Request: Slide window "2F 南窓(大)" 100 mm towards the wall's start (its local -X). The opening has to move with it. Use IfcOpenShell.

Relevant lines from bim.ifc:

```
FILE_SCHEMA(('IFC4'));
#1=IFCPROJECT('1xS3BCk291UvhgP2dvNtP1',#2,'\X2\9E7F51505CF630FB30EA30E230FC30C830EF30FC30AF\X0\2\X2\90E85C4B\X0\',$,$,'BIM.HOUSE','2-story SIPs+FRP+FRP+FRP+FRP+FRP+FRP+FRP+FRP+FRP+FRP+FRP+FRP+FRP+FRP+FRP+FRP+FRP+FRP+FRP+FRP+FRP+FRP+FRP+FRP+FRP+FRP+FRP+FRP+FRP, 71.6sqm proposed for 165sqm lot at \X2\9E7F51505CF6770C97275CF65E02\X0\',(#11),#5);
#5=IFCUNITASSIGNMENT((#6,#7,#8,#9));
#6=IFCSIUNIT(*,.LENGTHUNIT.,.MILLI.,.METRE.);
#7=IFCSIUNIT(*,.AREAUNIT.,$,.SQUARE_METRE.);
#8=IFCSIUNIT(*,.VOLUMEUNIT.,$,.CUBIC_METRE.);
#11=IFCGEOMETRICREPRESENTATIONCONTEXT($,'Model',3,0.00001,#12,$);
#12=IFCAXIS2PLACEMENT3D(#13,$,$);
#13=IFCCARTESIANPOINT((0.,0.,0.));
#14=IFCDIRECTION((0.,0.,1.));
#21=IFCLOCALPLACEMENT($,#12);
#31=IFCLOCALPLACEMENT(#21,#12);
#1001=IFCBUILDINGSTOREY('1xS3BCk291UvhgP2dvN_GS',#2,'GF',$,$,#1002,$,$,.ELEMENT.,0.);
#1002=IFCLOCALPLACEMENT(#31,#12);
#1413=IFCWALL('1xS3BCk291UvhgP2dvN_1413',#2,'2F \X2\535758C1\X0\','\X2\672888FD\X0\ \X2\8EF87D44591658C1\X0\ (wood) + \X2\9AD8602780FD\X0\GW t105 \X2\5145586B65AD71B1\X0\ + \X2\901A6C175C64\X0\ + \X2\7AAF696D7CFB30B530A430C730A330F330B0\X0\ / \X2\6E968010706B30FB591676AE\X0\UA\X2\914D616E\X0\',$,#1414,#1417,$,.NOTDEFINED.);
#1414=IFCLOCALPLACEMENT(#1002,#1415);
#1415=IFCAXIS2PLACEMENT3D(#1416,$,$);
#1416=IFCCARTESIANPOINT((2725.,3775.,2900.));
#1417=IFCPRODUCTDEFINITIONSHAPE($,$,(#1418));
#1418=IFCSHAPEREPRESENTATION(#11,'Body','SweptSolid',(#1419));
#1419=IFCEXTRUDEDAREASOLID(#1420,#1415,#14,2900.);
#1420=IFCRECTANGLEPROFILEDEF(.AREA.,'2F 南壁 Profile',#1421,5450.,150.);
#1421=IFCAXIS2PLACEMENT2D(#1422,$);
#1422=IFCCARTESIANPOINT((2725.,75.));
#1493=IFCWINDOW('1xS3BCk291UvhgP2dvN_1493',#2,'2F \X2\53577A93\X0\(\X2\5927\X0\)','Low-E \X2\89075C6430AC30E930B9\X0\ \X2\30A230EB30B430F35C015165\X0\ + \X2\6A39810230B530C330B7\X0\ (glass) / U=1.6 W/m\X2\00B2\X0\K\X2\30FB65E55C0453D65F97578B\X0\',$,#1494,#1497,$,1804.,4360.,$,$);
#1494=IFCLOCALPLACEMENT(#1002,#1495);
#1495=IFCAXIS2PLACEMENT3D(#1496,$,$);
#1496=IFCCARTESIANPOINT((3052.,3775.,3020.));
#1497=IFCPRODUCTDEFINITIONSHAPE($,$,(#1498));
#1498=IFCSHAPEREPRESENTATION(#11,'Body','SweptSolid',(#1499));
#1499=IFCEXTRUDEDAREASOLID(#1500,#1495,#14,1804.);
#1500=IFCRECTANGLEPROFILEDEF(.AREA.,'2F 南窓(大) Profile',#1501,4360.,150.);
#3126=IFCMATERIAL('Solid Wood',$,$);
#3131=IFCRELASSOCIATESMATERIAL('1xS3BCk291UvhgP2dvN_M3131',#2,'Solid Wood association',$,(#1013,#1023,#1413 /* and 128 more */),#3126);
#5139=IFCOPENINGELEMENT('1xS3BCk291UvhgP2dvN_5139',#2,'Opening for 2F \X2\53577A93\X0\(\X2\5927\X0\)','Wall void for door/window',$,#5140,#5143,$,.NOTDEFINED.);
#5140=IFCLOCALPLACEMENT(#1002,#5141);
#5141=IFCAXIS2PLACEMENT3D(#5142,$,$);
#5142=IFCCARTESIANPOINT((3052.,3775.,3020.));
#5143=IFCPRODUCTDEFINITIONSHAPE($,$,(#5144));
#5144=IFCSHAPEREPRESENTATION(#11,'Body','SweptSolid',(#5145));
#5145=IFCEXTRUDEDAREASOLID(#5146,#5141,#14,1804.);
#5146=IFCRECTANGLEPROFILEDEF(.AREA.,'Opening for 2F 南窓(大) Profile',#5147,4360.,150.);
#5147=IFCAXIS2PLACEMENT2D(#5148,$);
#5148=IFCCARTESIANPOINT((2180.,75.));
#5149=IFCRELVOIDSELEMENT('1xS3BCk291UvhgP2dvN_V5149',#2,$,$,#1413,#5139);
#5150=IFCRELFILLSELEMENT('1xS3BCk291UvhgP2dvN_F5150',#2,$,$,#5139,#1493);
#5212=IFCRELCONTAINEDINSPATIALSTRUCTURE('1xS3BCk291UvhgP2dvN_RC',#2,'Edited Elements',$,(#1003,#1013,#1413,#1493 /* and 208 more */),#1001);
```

```python
import ifcopenshell
import ifcopenshell.api.geometry
import ifcopenshell.util.placement

model = ifcopenshell.open("bim.ifc")

window = model.by_guid("1xS3BCk291UvhgP2dvN_1493")
opening = window.FillsVoids[0].RelatingOpeningElement
wall = opening.VoidsElements[0].RelatingBuildingElement

wall_matrix = ifcopenshell.util.placement.get_local_placement(wall.ObjectPlacement)
shift = wall_matrix[:3, 0] * -100.0
before = ifcopenshell.util.placement.get_local_placement(window.ObjectPlacement)[:3, 3].copy()

# The window is not placed relative to its opening, so move both.
for product in (opening, window):
    matrix = ifcopenshell.util.placement.get_local_placement(product.ObjectPlacement)
    matrix[:3, 3] += shift
    ifcopenshell.api.geometry.edit_object_placement(model, product=product, matrix=matrix, is_si=False)

after = ifcopenshell.util.placement.get_local_placement(window.ObjectPlacement)[:3, 3]
print("window moved by", (after - before).round(3) + 0.0)

model.write("bim_v2.ifc")
```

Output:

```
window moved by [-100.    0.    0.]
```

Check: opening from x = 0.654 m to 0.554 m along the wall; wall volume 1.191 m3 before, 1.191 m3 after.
